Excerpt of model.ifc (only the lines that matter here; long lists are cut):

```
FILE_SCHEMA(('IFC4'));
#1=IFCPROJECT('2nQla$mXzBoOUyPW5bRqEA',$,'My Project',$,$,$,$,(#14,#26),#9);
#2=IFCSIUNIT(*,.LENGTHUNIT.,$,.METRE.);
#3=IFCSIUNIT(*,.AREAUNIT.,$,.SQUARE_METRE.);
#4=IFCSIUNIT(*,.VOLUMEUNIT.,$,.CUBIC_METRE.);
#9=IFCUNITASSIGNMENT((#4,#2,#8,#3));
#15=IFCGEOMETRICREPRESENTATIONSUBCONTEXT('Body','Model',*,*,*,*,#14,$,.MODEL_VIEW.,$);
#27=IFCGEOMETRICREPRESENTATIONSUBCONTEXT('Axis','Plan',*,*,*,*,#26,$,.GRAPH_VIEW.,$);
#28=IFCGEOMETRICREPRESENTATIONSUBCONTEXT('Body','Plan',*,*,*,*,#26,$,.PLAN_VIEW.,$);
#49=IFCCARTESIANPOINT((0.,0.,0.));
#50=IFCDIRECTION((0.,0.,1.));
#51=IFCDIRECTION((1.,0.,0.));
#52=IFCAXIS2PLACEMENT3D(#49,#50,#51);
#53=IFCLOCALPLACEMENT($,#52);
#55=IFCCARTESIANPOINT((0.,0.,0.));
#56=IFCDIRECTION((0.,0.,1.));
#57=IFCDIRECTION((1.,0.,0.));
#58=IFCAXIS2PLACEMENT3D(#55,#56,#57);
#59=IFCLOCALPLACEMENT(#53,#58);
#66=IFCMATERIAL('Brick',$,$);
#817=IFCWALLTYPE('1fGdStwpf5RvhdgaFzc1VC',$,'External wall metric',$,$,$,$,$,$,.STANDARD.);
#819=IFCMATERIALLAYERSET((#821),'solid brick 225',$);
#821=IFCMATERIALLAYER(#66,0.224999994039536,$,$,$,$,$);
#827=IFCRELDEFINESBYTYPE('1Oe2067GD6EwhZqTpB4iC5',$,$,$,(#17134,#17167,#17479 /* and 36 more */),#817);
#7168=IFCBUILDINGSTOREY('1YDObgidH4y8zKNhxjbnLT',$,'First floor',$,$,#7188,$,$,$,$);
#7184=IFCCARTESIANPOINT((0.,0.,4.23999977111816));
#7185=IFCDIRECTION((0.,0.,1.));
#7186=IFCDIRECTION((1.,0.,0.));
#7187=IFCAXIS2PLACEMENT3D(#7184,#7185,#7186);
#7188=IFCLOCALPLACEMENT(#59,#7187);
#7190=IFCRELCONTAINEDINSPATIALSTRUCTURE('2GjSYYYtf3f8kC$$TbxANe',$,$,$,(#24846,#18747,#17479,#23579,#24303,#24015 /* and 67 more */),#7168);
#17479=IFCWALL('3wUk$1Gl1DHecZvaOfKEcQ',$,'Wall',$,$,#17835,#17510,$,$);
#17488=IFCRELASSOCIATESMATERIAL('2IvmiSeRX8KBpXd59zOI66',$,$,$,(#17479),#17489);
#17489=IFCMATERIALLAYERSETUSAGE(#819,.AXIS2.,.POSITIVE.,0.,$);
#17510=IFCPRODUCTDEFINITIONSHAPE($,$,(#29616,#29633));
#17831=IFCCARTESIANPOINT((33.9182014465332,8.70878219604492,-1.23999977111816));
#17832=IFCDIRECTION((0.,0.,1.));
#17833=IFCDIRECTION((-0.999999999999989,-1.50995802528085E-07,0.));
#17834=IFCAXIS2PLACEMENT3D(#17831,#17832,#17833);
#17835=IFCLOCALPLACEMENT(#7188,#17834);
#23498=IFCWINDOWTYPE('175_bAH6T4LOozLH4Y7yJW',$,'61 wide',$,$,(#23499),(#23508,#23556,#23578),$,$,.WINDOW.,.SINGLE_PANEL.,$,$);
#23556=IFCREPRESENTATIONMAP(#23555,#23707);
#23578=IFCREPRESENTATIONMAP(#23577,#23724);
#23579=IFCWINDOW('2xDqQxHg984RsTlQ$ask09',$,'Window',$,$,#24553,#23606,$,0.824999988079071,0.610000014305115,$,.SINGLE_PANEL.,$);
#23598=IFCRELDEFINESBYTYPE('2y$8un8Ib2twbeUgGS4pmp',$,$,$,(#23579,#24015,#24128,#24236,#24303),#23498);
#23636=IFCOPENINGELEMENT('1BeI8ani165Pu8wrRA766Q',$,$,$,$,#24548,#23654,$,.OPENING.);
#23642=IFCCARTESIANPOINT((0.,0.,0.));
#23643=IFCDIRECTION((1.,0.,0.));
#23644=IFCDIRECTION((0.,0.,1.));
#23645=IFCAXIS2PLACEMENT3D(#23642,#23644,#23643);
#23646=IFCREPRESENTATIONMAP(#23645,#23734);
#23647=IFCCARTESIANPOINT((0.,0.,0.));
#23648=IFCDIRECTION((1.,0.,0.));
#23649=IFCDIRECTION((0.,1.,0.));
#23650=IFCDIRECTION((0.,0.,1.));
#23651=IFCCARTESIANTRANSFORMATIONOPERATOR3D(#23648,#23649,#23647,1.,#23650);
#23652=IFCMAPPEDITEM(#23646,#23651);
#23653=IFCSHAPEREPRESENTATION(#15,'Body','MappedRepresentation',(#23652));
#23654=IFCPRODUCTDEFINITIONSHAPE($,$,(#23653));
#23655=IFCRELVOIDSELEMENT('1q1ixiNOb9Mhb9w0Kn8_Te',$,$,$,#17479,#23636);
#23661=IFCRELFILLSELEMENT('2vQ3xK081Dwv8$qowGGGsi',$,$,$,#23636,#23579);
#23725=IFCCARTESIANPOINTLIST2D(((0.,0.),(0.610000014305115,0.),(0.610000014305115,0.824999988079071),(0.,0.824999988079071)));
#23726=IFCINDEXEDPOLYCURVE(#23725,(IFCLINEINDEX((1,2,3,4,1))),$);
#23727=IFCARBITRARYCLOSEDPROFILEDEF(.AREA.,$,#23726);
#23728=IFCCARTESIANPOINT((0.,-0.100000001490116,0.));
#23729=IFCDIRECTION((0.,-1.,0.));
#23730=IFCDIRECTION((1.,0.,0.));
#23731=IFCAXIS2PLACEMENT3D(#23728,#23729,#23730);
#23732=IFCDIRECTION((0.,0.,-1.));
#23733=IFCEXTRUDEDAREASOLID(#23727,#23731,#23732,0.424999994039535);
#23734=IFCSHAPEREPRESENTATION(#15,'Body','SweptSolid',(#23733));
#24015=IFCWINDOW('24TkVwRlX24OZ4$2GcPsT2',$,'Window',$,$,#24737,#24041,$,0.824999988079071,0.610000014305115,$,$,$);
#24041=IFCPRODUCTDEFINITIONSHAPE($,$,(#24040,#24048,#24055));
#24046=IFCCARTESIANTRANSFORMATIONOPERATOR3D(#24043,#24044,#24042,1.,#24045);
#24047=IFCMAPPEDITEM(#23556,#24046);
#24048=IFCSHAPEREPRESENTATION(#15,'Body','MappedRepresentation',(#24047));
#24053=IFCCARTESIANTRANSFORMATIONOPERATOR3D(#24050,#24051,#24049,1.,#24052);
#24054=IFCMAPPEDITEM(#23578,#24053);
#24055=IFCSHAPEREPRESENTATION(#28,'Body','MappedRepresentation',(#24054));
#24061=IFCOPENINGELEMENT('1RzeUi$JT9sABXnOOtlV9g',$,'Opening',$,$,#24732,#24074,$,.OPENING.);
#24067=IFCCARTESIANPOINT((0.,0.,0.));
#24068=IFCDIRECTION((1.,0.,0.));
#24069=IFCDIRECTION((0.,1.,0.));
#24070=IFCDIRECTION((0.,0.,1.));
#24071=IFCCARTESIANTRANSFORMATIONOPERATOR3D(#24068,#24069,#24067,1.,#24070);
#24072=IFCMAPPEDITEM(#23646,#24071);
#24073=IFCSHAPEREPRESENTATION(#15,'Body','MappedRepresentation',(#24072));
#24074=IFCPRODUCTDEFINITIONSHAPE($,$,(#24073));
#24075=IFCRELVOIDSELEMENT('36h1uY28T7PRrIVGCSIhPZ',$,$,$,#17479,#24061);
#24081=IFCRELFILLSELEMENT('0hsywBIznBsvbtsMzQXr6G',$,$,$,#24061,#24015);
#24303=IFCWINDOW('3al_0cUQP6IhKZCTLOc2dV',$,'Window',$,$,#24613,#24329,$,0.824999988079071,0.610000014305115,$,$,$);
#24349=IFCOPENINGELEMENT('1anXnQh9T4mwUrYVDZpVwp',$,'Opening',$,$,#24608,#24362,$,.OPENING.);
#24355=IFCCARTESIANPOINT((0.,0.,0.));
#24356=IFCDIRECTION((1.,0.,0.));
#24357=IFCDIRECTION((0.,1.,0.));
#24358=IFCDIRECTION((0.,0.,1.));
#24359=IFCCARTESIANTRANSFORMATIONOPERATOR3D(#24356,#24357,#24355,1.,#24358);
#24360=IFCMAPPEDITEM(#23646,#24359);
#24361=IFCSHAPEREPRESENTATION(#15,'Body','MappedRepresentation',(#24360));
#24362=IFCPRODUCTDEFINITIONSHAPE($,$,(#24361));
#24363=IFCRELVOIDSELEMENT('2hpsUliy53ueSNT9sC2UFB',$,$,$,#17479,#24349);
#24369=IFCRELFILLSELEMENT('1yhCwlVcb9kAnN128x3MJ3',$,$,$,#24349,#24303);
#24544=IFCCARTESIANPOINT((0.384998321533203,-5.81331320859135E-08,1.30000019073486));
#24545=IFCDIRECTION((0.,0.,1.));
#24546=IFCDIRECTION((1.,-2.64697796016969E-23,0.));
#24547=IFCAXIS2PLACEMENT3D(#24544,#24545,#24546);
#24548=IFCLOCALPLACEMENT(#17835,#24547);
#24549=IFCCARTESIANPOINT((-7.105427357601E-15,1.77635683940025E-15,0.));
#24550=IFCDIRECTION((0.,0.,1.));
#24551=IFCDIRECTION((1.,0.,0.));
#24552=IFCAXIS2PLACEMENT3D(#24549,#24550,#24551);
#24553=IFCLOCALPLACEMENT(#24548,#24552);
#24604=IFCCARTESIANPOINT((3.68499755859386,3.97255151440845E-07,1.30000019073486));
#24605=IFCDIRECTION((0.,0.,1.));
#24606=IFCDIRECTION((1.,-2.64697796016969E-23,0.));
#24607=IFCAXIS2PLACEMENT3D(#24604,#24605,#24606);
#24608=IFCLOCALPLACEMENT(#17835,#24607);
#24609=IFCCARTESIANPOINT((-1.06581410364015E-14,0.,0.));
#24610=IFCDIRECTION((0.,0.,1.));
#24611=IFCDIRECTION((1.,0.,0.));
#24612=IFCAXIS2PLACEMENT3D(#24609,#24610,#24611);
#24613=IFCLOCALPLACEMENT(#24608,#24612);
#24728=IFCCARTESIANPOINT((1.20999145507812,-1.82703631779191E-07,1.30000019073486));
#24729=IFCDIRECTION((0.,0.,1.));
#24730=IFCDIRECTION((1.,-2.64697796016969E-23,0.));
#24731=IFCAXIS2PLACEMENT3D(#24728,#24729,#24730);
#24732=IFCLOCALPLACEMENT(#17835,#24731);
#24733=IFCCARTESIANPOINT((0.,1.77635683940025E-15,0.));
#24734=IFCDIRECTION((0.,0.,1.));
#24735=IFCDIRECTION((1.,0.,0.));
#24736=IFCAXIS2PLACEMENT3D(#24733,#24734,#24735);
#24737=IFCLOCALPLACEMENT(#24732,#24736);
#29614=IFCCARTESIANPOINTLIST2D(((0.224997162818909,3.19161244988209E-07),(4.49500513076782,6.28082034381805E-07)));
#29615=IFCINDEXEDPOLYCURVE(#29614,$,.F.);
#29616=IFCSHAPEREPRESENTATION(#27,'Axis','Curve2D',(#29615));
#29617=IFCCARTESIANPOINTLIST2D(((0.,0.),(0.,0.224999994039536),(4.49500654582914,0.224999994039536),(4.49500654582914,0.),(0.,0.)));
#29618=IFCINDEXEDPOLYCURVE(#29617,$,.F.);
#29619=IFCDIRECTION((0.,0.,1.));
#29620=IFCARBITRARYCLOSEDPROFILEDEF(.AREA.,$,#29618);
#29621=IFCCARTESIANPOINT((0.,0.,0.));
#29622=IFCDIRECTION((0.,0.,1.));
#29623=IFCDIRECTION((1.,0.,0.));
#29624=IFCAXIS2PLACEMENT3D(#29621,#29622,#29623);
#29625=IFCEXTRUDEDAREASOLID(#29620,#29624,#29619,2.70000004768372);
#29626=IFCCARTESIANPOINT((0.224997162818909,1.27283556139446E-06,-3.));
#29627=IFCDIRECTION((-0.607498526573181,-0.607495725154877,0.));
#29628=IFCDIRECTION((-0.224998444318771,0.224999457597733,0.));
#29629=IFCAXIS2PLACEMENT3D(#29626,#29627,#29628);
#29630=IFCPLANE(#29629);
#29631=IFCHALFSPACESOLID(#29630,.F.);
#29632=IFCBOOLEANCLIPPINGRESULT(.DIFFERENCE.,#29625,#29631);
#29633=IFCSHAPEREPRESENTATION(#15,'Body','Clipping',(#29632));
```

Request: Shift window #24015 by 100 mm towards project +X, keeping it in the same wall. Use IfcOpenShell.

```python
import ifcopenshell
import ifcopenshell.api.geometry
import ifcopenshell.util.placement
import ifcopenshell.util.unit

model = ifcopenshell.open("model.ifc")
unit_scale = ifcopenshell.util.unit.calculate_unit_scale(model)

window = model.by_guid("24TkVwRlX24OZ4$2GcPsT2")
opening = window.FillsVoids[0].RelatingOpeningElement
wall = opening.VoidsElements[0].RelatingBuildingElement

wall_matrix = ifcopenshell.util.placement.get_local_placement(wall.ObjectPlacement)
shift = wall_matrix[:3, 0] * -0.1 / unit_scale
before = ifcopenshell.util.placement.get_local_placement(window.ObjectPlacement)[:3, 3].copy()

# The window is placed relative to its opening, so it follows when the opening moves.
matrix = ifcopenshell.util.placement.get_local_placement(opening.ObjectPlacement)
matrix[:3, 3] += shift
ifcopenshell.api.geometry.edit_object_placement(
    model, product=opening, matrix=matrix, is_si=False, should_transform_children=True
)

after = ifcopenshell.util.placement.get_local_placement(window.ObjectPlacement)[:3, 3]
print("window moved by", (after - before).round(3) + 0.0)

model.write("model_v2.ifc")
```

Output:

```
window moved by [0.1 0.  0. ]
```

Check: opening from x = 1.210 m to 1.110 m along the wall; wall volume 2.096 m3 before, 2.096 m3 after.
